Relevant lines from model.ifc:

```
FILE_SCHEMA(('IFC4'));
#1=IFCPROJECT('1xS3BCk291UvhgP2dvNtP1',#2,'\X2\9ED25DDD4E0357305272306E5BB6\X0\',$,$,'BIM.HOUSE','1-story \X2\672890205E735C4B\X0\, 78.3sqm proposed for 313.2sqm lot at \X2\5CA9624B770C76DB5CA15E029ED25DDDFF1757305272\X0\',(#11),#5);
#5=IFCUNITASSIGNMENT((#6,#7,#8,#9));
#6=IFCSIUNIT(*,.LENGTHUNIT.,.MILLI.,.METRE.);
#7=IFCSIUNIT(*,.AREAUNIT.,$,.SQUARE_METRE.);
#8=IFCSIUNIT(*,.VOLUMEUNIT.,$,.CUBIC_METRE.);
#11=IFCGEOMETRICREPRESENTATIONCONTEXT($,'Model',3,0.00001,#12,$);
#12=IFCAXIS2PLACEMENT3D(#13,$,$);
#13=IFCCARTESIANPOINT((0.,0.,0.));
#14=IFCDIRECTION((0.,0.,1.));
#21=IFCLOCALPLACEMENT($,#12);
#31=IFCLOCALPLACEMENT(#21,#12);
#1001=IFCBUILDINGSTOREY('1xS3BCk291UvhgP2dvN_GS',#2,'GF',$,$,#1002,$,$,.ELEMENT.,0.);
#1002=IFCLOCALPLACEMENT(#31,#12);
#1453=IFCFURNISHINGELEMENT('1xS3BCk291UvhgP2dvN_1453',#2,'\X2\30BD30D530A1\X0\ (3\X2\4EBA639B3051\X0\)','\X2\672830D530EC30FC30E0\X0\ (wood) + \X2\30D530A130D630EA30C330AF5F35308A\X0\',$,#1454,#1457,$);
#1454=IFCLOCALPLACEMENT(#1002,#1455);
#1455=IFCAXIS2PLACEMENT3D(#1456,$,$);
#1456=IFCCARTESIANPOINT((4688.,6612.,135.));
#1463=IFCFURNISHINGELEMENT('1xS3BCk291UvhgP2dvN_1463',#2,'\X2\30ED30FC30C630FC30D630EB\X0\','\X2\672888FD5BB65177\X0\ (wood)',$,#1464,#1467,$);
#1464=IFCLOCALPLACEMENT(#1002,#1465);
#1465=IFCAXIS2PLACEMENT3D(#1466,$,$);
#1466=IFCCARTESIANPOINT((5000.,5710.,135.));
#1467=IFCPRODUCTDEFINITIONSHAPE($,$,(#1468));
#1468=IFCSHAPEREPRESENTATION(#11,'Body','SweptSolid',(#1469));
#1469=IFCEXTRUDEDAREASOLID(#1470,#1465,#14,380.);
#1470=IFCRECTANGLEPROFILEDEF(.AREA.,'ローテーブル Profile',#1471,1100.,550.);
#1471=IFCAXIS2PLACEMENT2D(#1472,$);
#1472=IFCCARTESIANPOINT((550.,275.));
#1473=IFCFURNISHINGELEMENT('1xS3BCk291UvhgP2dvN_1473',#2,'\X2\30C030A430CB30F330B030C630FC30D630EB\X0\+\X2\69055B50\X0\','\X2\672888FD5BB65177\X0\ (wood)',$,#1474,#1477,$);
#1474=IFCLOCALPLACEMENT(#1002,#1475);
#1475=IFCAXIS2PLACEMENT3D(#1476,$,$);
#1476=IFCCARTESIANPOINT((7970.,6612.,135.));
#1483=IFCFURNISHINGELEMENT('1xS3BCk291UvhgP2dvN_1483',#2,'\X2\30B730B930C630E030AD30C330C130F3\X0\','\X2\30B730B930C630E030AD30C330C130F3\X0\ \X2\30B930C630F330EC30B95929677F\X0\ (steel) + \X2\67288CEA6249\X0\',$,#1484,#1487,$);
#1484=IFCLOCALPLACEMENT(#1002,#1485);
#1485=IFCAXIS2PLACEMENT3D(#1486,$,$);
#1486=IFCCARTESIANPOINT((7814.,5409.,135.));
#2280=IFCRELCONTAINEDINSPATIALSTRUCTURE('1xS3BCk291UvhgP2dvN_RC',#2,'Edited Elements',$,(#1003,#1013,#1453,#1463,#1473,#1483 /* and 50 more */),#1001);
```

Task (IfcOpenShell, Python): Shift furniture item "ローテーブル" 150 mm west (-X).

```python
import ifcopenshell
import ifcopenshell.api.geometry
import ifcopenshell.util.placement

model = ifcopenshell.open("model.ifc")

item = model.by_guid("1xS3BCk291UvhgP2dvN_1463")
matrix = ifcopenshell.util.placement.get_local_placement(item.ObjectPlacement)
matrix[0, 3] -= 150.0
ifcopenshell.api.geometry.edit_object_placement(model, product=item, matrix=matrix, is_si=False)

print(ifcopenshell.util.placement.get_local_placement(item.ObjectPlacement).round(3) + 0.0)

model.write("model_edited.ifc")
```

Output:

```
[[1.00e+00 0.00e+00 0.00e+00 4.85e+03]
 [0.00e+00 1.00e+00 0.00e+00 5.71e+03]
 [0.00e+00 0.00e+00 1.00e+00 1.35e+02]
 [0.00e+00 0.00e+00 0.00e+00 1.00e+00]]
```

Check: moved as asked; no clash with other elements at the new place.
